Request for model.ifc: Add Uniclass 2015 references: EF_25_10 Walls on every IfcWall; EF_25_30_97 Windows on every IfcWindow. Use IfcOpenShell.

First a look at what the model holds.

```python
import ifcopenshell

model = ifcopenshell.open("model.ifc")
print(model.schema)
print("classifications:", [c.Name for c in model.by_type("IfcClassification")])
for ifc_class in ("IfcDoor", "IfcRoof", "IfcStair", "IfcWall", "IfcWindow"):
    print(ifc_class, len(model.by_type(ifc_class)))
```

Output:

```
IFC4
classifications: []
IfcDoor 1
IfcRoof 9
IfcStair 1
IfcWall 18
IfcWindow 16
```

```python
import ifcopenshell
import ifcopenshell.api.classification

model = ifcopenshell.open("model.ifc")

system = ifcopenshell.api.classification.add_classification(model, classification="Uniclass 2015")

codes = {
    "IfcWall": ("EF_25_10", "Walls"),
    "IfcWindow": ("EF_25_30_97", "Windows"),
}
for ifc_class, (code, name) in codes.items():
    products = model.by_type(ifc_class)
    ifcopenshell.api.classification.add_reference(
        model, products=products, classification=system, identification=code, name=name
    )
    print(code, len(products))

model.write("model_edited.ifc")
```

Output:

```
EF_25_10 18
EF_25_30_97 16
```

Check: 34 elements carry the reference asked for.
